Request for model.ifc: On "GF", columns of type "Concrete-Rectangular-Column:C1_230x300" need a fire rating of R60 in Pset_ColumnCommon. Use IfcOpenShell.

First a look at what the model holds.

```python
import ifcopenshell
import ifcopenshell.util.element

model = ifcopenshell.open("model.ifc")
print(model.schema)
storey = next(s for s in model.by_type("IfcBuildingStorey") if s.Name == "GF")
columns = [e for e in ifcopenshell.util.element.get_decomposition(storey) if e.is_a("IfcColumn")]
seen = {}
for e in columns:
    element_type = ifcopenshell.util.element.get_type(e)
    key = (element_type.Name if element_type != e and element_type else None, ifcopenshell.util.element.get_pset(e, "Pset_ColumnCommon", "FireRating"))
    seen[key] = seen.get(key, 0) + 1
for (name, value), count in sorted(seen.items(), key=str):
    print(count, "x", name, "|", value)
```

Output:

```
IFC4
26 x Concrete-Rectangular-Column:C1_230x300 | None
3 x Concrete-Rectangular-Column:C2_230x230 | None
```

```python
import ifcopenshell
import ifcopenshell.api.pset
import ifcopenshell.util.element

model = ifcopenshell.open("model.ifc")

storey = next(s for s in model.by_type("IfcBuildingStorey") if s.Name == "GF")
columns = [e for e in ifcopenshell.util.element.get_decomposition(storey) if e.is_a("IfcColumn")]

count = 0
for e in columns:
    element_type = ifcopenshell.util.element.get_type(e)
    if element_type in (None, e) or element_type.Name != "Concrete-Rectangular-Column:C1_230x300":
        continue
    # add_pset returns the element's existing set when there is one.
    pset = ifcopenshell.api.pset.add_pset(model, product=e, name="Pset_ColumnCommon")
    ifcopenshell.api.pset.edit_pset(model, pset=pset, properties={"FireRating": "R60"})
    count += 1

print(count, "columns updated")

model.write("model-out.ifc")
```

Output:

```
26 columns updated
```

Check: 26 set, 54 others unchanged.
